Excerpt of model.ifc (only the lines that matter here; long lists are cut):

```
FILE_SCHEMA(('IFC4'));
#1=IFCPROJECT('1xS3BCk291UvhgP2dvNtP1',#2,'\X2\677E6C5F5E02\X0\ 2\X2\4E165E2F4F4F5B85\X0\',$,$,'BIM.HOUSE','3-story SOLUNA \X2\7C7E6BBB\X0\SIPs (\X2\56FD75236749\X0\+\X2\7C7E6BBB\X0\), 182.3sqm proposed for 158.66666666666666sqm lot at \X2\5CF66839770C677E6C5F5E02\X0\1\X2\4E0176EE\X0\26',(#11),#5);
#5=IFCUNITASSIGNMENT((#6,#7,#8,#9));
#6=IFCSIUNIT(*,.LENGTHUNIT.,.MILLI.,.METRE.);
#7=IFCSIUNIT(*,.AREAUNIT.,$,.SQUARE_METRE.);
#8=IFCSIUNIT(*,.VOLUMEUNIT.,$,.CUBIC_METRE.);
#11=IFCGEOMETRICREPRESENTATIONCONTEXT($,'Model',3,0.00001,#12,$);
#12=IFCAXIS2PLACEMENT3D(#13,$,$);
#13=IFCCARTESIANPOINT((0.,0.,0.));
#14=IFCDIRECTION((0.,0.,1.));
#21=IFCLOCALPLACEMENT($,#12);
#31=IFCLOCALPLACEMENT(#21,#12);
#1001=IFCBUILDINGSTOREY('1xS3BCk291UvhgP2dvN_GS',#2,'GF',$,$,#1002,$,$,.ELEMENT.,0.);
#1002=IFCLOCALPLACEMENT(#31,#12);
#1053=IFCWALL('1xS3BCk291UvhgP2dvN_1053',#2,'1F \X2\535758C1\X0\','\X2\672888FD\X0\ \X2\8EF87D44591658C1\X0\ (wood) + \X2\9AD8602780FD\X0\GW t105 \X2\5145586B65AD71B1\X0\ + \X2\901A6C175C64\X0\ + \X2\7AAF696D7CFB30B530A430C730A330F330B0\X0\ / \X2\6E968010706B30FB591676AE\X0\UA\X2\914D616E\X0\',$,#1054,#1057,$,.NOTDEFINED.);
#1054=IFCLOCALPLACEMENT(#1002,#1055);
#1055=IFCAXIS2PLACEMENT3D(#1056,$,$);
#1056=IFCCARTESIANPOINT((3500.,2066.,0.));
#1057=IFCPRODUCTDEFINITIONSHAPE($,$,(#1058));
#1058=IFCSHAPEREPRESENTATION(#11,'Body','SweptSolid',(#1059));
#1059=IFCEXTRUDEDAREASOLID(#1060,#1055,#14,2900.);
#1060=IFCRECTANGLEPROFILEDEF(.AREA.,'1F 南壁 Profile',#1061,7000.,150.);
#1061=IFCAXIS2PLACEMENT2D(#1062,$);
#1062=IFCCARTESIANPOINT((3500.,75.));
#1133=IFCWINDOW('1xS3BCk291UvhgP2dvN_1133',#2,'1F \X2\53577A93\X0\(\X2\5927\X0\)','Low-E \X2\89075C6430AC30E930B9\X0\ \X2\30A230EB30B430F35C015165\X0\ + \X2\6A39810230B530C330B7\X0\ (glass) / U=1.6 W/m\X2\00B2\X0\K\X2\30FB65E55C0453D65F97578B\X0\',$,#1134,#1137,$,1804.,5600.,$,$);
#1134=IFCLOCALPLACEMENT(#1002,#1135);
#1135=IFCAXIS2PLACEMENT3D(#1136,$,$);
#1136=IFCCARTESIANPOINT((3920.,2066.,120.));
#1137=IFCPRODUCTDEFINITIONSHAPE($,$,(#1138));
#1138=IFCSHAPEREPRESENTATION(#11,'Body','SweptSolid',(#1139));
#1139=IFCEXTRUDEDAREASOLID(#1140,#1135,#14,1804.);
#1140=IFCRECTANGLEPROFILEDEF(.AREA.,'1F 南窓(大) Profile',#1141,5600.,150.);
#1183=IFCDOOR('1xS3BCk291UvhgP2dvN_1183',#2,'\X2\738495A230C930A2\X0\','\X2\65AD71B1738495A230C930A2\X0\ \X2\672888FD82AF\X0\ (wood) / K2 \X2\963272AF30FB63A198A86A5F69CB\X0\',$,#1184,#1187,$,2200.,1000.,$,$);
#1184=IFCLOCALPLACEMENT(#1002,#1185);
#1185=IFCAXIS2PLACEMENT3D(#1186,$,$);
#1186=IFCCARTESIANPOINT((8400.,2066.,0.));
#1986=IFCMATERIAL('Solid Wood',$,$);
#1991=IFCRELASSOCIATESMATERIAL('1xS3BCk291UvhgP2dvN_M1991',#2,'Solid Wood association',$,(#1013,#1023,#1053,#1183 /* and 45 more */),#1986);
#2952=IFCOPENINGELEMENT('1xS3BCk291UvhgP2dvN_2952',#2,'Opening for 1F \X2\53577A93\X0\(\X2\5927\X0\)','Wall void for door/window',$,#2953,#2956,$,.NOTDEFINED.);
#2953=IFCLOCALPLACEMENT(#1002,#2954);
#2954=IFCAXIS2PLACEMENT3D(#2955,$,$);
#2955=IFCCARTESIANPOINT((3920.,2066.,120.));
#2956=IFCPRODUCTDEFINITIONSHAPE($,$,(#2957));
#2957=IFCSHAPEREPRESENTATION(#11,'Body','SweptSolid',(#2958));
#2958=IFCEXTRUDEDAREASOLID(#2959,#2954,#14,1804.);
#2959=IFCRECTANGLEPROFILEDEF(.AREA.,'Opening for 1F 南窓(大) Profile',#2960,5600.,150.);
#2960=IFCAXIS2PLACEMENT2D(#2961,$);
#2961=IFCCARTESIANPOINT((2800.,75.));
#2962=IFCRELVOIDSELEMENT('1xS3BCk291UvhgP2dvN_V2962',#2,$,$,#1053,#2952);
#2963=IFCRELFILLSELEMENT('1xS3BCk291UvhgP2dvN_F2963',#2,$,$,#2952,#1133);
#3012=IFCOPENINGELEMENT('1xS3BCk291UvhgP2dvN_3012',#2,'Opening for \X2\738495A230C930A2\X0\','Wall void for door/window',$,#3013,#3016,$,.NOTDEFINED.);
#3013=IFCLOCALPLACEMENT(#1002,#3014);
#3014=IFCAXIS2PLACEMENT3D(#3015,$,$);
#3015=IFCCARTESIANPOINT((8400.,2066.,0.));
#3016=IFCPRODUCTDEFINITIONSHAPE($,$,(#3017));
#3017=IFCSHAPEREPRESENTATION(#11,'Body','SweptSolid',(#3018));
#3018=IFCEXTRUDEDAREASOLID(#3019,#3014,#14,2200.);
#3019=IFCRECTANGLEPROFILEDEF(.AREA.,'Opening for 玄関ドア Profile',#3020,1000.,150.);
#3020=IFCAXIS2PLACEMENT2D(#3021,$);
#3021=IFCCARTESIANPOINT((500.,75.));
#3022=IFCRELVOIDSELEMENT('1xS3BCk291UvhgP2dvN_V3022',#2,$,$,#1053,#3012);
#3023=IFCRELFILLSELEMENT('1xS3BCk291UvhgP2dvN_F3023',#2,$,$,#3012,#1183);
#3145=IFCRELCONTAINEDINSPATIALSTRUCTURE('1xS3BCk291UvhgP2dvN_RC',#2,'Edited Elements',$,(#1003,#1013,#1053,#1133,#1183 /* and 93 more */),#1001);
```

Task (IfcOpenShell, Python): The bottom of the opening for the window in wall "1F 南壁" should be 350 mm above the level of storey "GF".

```python
import numpy as np
import ifcopenshell
import ifcopenshell.api.geometry
import ifcopenshell.geom
import ifcopenshell.util.element
import ifcopenshell.util.placement
import ifcopenshell.util.shape
import ifcopenshell.util.unit

model = ifcopenshell.open("model.ifc")
unit_scale = ifcopenshell.util.unit.calculate_unit_scale(model)

window = model.by_guid("1xS3BCk291UvhgP2dvN_1133")
opening = window.FillsVoids[0].RelatingOpeningElement
storey = ifcopenshell.util.element.get_container(window, ifc_class="IfcBuildingStorey")
level = ifcopenshell.util.placement.get_local_placement(storey.ObjectPlacement)[2, 3]

# The opening's origin need not be at the sill, so measure its lowest point.
shape = ifcopenshell.geom.create_shape(ifcopenshell.geom.settings(), opening)
bottom = ifcopenshell.util.shape.get_shape_bottom_elevation(shape, shape.geometry) / unit_scale
dz = level + 0.35 / unit_scale - bottom

shift = np.array([0.0, 0.0, dz])
# The window is not placed relative to its opening, so move both.
for product in (opening, window):
    matrix = ifcopenshell.util.placement.get_local_placement(product.ObjectPlacement)
    matrix[:3, 3] += shift
    ifcopenshell.api.geometry.edit_object_placement(model, product=product, matrix=matrix, is_si=False)

print(f"moved by {dz * unit_scale:+.3f} m")

model.write("model_edited.ifc")
```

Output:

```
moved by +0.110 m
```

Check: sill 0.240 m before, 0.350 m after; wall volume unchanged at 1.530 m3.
